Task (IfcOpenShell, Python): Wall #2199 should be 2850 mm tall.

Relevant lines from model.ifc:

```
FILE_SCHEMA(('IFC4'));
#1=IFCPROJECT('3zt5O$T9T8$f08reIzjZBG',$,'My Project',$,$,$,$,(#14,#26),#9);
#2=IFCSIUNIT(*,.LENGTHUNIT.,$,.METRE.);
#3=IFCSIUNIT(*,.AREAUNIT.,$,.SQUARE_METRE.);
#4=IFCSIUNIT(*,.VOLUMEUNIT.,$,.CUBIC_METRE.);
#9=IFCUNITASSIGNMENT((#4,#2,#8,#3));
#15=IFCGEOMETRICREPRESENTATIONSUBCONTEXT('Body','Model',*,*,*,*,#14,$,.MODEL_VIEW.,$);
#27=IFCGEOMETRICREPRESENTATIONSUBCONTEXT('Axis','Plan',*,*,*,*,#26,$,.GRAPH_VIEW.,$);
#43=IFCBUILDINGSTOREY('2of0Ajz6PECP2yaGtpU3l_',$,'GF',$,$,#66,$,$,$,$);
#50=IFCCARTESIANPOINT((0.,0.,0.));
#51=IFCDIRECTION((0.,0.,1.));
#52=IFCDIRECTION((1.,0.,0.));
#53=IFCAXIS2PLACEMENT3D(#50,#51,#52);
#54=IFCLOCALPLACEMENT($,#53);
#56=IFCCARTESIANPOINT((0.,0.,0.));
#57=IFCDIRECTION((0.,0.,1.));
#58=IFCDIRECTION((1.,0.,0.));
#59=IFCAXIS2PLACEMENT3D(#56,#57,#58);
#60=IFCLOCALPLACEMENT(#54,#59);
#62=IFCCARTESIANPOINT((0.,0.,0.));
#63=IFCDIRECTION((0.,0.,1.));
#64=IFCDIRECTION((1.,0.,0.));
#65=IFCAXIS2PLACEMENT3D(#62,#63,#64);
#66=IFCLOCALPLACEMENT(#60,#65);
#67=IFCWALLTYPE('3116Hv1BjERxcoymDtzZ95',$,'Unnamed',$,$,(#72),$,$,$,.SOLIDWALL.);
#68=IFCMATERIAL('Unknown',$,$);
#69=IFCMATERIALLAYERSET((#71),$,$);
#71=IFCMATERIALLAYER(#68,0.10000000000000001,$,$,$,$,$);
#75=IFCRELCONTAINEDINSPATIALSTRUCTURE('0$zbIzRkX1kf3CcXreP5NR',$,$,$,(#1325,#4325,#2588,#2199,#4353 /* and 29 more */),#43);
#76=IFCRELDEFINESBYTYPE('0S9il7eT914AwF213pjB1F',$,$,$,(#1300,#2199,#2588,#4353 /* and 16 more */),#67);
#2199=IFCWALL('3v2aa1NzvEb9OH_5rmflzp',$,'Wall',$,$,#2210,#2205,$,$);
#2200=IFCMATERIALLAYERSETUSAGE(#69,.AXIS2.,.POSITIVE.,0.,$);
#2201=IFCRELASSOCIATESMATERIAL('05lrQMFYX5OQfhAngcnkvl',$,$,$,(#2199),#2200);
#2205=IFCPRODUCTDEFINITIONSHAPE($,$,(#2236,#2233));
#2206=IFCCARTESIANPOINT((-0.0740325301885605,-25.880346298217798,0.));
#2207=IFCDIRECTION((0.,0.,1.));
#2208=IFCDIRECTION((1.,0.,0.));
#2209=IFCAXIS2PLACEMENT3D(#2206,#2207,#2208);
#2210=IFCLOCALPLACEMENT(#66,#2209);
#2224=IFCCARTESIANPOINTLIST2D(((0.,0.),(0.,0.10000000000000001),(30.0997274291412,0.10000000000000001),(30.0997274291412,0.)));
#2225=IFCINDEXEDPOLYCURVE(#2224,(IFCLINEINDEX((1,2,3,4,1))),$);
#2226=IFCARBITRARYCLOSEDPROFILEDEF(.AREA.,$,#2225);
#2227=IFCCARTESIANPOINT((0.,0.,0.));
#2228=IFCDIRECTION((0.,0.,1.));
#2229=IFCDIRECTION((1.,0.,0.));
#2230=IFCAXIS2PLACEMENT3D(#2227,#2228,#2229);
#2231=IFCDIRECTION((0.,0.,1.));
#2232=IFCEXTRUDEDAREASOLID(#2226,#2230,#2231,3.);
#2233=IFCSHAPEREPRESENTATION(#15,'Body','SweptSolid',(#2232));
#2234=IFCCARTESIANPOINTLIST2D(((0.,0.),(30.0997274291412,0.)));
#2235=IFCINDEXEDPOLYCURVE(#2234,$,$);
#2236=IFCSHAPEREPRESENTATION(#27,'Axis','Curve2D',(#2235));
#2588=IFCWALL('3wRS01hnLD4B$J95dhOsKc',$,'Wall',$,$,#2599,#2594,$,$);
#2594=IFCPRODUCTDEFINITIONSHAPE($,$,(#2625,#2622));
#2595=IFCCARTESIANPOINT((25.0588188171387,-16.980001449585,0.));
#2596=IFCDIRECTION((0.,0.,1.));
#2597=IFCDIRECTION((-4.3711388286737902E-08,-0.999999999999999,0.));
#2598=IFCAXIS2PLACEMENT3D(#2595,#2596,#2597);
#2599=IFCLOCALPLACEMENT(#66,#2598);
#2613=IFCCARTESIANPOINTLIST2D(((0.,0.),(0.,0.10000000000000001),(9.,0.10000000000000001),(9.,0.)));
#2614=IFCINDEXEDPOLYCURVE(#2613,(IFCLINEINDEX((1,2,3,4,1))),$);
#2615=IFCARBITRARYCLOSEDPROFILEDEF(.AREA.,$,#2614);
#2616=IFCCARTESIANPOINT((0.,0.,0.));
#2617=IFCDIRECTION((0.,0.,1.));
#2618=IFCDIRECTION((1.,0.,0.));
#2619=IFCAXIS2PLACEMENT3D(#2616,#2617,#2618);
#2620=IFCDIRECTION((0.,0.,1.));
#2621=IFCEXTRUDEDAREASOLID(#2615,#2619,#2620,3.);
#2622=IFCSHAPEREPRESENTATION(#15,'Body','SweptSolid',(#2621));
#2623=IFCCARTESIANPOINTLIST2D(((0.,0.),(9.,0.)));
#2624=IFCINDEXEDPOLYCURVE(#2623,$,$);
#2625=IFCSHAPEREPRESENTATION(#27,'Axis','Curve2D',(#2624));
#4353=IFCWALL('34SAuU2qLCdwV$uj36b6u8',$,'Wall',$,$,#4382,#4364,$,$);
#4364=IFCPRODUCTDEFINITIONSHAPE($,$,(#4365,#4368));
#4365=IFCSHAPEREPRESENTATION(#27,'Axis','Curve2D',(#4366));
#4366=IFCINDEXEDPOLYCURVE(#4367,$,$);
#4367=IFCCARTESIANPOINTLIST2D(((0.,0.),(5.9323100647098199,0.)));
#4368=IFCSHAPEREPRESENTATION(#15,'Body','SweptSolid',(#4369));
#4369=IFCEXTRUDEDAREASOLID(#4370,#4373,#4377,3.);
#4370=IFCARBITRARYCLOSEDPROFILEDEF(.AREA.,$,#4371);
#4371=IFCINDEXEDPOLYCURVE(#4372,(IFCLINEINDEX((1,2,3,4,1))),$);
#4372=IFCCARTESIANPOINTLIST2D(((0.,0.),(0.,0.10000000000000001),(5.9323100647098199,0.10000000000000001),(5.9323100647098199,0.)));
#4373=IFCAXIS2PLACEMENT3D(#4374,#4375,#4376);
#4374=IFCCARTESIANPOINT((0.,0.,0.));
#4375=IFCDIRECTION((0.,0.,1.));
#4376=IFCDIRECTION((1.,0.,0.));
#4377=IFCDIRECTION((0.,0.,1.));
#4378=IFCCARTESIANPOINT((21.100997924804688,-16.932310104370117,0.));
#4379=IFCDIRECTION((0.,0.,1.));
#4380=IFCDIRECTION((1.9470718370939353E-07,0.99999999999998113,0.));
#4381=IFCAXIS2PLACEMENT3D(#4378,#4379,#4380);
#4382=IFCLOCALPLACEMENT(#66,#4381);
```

```python
import ifcopenshell
import ifcopenshell.geom
import ifcopenshell.util.representation
import ifcopenshell.util.shape
import ifcopenshell.util.unit

model = ifcopenshell.open("model.ifc")
unit_scale = ifcopenshell.util.unit.calculate_unit_scale(model)
settings = ifcopenshell.geom.settings()


def volume(element):
    """Net volume in cubic metres, openings subtracted."""
    shape = ifcopenshell.geom.create_shape(settings, element)
    return ifcopenshell.util.shape.get_volume(shape.geometry)


wall = model.by_id(2199)
before = volume(wall)

body = ifcopenshell.util.representation.get_representation(wall, "Model", "Body")
solid = body.Items[0]
old_height = solid.Depth
solid.Depth = 2.85 / unit_scale
after = volume(wall)

print(f"height {old_height:g} -> {solid.Depth:g}, volume {before:.3f} -> {after:.3f} m3")

model.write("model_edited.ifc")
```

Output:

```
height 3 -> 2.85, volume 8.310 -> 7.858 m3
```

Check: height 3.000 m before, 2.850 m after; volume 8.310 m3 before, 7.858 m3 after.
